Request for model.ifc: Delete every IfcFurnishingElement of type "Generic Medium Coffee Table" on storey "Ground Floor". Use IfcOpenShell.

First a look at what the model holds.

```python
import ifcopenshell
import ifcopenshell.util.element

model = ifcopenshell.open("model.ifc")
print(model.schema)
storey = next(s for s in model.by_type("IfcBuildingStorey") if s.Name == "Ground Floor")
furniture = [e for e in ifcopenshell.util.element.get_decomposition(storey) if e.is_a("IfcFurnishingElement")]
seen = {}
for e in furniture:
    element_type = ifcopenshell.util.element.get_type(e)
    name = element_type.Name if element_type not in (None, e) else None
    seen[name] = seen.get(name, 0) + 1
for name, count in sorted(seen.items(), key=str):
    print(count, "x", name)
```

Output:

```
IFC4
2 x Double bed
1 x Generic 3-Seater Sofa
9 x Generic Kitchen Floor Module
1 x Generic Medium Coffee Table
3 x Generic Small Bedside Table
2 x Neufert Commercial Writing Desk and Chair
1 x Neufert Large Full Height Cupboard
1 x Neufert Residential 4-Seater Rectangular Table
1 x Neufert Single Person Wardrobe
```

```python
import ifcopenshell
import ifcopenshell.api.root
import ifcopenshell.util.element

model = ifcopenshell.open("model.ifc")

storey = next(s for s in model.by_type("IfcBuildingStorey") if s.Name == "Ground Floor")
furniture = [e for e in ifcopenshell.util.element.get_decomposition(storey) if e.is_a("IfcFurnishingElement")]
targets = [e for e in furniture if (t := ifcopenshell.util.element.get_type(e)) not in (None, e) and t.Name == "Generic Medium Coffee Table"]

for e in targets:
    ifcopenshell.api.root.remove_product(model, product=e)
print(len(targets), "removed")

model.write("model-out.ifc")
```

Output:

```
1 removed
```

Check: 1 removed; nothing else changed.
